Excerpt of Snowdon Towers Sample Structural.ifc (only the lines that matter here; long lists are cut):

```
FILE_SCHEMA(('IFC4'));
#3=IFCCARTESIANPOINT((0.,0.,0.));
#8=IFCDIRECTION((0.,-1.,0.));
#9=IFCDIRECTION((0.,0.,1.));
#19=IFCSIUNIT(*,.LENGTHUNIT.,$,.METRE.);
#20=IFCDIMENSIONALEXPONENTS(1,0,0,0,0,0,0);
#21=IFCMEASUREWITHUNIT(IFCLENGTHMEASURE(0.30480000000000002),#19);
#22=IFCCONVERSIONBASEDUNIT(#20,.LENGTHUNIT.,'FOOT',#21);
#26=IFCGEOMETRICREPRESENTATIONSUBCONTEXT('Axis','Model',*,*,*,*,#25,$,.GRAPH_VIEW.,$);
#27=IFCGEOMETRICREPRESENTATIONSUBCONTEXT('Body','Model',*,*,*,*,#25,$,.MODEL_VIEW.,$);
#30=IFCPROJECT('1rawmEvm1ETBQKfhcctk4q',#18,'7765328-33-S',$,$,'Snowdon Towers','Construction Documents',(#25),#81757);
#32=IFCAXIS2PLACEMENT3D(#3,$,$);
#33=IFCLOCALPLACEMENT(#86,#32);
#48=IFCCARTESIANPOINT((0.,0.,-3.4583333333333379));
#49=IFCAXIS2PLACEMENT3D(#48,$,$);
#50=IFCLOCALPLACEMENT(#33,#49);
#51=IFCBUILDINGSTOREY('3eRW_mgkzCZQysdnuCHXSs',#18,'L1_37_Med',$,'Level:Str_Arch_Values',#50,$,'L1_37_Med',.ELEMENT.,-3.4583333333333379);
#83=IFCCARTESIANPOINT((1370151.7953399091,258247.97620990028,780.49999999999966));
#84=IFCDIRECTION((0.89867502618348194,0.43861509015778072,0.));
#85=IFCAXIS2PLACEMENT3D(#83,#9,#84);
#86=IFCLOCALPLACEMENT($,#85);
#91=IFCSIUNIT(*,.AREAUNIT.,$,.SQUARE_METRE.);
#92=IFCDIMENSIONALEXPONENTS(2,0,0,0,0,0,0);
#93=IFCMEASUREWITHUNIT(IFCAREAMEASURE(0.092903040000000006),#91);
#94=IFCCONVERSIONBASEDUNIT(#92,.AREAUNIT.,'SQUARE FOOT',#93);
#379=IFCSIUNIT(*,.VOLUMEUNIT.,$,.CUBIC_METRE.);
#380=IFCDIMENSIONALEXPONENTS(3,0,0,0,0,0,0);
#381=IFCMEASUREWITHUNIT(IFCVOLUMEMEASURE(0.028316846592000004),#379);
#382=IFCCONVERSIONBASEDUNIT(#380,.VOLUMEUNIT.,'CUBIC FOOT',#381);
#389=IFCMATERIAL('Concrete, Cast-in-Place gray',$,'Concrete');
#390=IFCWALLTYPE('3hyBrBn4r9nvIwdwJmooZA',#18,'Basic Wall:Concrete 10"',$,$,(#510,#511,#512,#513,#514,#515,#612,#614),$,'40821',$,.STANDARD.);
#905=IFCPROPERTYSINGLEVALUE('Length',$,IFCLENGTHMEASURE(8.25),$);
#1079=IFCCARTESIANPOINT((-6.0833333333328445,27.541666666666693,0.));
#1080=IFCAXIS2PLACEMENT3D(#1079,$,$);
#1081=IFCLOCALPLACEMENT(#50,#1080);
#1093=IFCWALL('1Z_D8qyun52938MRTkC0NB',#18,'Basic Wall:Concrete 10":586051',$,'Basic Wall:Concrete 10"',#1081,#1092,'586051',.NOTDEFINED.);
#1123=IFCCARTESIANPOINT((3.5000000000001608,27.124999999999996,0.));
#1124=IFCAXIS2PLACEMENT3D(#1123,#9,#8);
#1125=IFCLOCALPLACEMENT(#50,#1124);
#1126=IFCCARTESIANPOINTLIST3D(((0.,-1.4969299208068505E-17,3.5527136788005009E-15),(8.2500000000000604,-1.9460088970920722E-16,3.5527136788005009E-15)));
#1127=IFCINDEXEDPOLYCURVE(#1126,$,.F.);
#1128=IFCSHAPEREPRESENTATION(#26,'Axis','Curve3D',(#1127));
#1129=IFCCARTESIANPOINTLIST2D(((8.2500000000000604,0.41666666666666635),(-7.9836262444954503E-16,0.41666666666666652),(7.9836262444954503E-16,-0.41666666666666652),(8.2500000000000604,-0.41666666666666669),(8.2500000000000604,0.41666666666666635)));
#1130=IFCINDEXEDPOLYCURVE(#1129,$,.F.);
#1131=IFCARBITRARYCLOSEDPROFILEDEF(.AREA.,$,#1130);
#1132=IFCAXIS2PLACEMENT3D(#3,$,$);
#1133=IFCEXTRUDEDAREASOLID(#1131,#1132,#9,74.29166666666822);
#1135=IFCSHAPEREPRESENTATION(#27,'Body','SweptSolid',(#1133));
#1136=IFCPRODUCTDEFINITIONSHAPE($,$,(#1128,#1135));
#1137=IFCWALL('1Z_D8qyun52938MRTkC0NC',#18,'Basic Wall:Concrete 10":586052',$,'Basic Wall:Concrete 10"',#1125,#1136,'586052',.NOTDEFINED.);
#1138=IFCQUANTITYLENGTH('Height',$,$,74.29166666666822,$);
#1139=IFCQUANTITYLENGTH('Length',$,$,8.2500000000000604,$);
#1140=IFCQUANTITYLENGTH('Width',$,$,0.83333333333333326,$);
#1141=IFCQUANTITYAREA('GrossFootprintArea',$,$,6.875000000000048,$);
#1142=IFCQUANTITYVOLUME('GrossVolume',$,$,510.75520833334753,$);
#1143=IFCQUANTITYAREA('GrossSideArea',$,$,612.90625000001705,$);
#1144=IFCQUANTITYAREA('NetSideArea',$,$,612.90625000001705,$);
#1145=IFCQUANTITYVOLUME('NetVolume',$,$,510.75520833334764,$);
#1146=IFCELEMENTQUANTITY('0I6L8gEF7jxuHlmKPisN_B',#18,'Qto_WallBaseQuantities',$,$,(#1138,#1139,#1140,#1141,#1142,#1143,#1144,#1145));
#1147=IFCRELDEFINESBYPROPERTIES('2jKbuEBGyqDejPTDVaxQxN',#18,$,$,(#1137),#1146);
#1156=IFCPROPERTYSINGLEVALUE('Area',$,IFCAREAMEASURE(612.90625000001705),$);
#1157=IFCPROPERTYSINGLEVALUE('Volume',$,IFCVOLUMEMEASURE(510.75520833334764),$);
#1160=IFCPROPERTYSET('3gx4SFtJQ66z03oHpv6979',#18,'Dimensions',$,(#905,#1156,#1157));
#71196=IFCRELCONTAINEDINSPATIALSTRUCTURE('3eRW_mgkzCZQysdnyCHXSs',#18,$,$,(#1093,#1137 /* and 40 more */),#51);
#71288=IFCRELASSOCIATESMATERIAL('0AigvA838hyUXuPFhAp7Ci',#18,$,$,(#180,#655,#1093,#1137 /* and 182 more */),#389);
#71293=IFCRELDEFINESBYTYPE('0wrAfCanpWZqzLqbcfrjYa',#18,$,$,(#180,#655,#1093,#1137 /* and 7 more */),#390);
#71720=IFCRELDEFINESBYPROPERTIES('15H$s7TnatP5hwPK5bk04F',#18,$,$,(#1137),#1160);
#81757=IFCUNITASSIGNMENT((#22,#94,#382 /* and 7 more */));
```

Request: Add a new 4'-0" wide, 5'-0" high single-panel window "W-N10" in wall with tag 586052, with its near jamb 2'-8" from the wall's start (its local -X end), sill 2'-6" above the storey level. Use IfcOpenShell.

```python
import numpy as np
import ifcopenshell
import ifcopenshell.api.feature
import ifcopenshell.api.geometry
import ifcopenshell.api.pset
import ifcopenshell.api.root
import ifcopenshell.api.spatial
import ifcopenshell.geom
import ifcopenshell.util.element
import ifcopenshell.util.placement
import ifcopenshell.util.representation
import ifcopenshell.util.shape
import ifcopenshell.util.unit

model = ifcopenshell.open("Snowdon Towers Sample Structural.ifc")
unit_scale = ifcopenshell.util.unit.calculate_unit_scale(model)
area_scale = ifcopenshell.util.unit.calculate_unit_scale(model, "AREAUNIT")
volume_scale = ifcopenshell.util.unit.calculate_unit_scale(model, "VOLUMEUNIT")
settings = ifcopenshell.geom.settings()


def volume(element):
    """Net volume in cubic metres, openings subtracted."""
    shape = ifcopenshell.geom.create_shape(settings, element)
    return ifcopenshell.util.shape.get_volume(shape.geometry)


wall = model.by_guid("1Z_D8qyun52938MRTkC0NC")
storey = ifcopenshell.util.element.get_container(wall, ifc_class="IfcBuildingStorey")
context = ifcopenshell.util.representation.get_context(model, "Model", "Body", "MODEL_VIEW")
before = volume(wall)

width, height, from_end, sill = 1.2192, 1.524, 0.8128, 0.762  # metres

# The wall runs along its own X axis, and the end named is its -X end.
wall_shape = ifcopenshell.geom.create_shape(settings, wall)
x, y, z = ifcopenshell.util.shape.get_vertices(wall_shape.geometry).T
start = x.min() + from_end
face, thickness = float(y.min()), float(y.max() - y.min())
wall_matrix = ifcopenshell.util.placement.get_local_placement(wall.ObjectPlacement)
level = ifcopenshell.util.placement.get_local_placement(storey.ObjectPlacement)[2, 3]


def in_wall(x, y):
    """Placement at x, y metres in the wall's axes, at sill height."""
    matrix = wall_matrix.copy()
    matrix[:, 3] = wall_matrix @ np.array([x / unit_scale, y / unit_scale, 0.0, 1.0])
    matrix[2, 3] = level + sill / unit_scale
    return matrix


# Opening: a box that overshoots both wall faces by 50 mm.
opening = ifcopenshell.api.root.create_entity(model, ifc_class="IfcOpeningElement", predefined_type="OPENING")
box = ifcopenshell.api.geometry.add_wall_representation(
    model, context=context, length=width, height=height, thickness=thickness + 0.1
)
ifcopenshell.api.geometry.assign_representation(model, product=opening, representation=box)
ifcopenshell.api.geometry.edit_object_placement(model, product=opening, matrix=in_wall(start, face - 0.05), is_si=False)
ifcopenshell.api.feature.add_feature(model, feature=opening, element=wall)

window = ifcopenshell.api.root.create_entity(model, ifc_class="IfcWindow", name="W-N10", predefined_type="WINDOW")
window.OverallWidth, window.OverallHeight = width / unit_scale, height / unit_scale
window.PartitioningType = "SINGLE_PANEL"
body = ifcopenshell.api.geometry.add_window_representation(
    model,
    context=context,
    overall_width=window.OverallWidth,
    overall_height=window.OverallHeight,
    partition_type="SINGLE_PANEL",
)
ifcopenshell.api.geometry.assign_representation(model, product=window, representation=body)
ifcopenshell.api.spatial.assign_container(model, products=[window], relating_structure=storey)
ifcopenshell.api.feature.add_filling(model, opening=opening, element=window)

# Centre the window in the wall's thickness.
ifcopenshell.api.geometry.edit_object_placement(model, product=window, matrix=in_wall(start, face), is_si=False)
window_shape = ifcopenshell.geom.create_shape(settings, window)
depth = ifcopenshell.util.shape.get_vertices(window_shape.geometry)[:, 1]
offset = face + thickness / 2 - (depth.min() + depth.max()) / 2
ifcopenshell.api.geometry.edit_object_placement(model, product=window, matrix=in_wall(start, offset), is_si=False)

after = volume(wall)

# Update the wall's stored quantities.
qto = model.by_id(ifcopenshell.util.element.get_pset(wall, "Qto_WallBaseQuantities", should_inherit=False)["id"])
ifcopenshell.api.pset.edit_qto(model, qto=qto, properties={
    "NetSideArea": after / thickness / area_scale,
    "NetVolume": after / volume_scale,
})
pset = model.by_id(ifcopenshell.util.element.get_pset(wall, "Dimensions", should_inherit=False)["id"])
ifcopenshell.api.pset.edit_pset(model, pset=pset, properties={
    "Area": model.create_entity("IfcAreaMeasure", after / thickness / area_scale),
    "Volume": model.create_entity("IfcVolumeMeasure", after / volume_scale),
})

print(f"wall volume {before:.3f} -> {after:.3f} m3")

model.write("Snowdon Towers Sample Structural_v2.ifc")
```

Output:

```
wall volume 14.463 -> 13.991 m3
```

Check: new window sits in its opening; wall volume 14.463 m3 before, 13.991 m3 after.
